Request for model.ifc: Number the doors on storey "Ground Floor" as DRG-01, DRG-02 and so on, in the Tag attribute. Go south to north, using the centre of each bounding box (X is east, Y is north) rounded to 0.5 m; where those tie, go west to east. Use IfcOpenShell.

First a look at what the model holds.

```python
import ifcopenshell
import ifcopenshell.util.element
import ifcopenshell.util.placement

model = ifcopenshell.open("model.ifc")
print(model.schema)
storey = next(s for s in model.by_type("IfcBuildingStorey") if s.Name == "Ground Floor")
doors = [e for e in ifcopenshell.util.element.get_decomposition(storey) if e.is_a("IfcDoor")]
for e in sorted(doors, key=lambda e: e.id()):
    origin = ifcopenshell.util.placement.get_local_placement(e.ObjectPlacement)[:3, 3]
    print(e.id(), e.Tag, e.Name, origin.round(2) + 0.0, sep=" | ")
```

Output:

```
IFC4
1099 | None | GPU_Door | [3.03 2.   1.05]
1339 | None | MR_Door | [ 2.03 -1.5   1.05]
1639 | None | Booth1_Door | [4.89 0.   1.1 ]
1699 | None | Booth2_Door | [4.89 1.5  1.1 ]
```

```python
import ifcopenshell
import ifcopenshell.geom
import ifcopenshell.util.element
import ifcopenshell.util.shape

model = ifcopenshell.open("model.ifc")
settings = ifcopenshell.geom.settings()
settings.set("use-world-coords", True)


def centre(element):
    shape = ifcopenshell.geom.create_shape(settings, element)
    return ifcopenshell.util.shape.get_bbox_centroid(shape.geometry)


storey = next(s for s in model.by_type("IfcBuildingStorey") if s.Name == "Ground Floor")
doors = [e for e in ifcopenshell.util.element.get_decomposition(storey) if e.is_a("IfcDoor")]

# Insertion points can sit at a corner or the storey origin, so sort by the geometry (in metres).
centres = {e: centre(e) for e in doors}
doors.sort(key=lambda e: (round(centres[e][1] / 0.5), centres[e][0]))

for i, e in enumerate(doors, start=1):
    number = f"DRG-{i:02d}"
    e.Tag = number
    print(e.id(), number)

model.write("model_updated.ifc")
```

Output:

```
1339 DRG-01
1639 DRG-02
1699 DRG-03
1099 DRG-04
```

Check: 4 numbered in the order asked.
